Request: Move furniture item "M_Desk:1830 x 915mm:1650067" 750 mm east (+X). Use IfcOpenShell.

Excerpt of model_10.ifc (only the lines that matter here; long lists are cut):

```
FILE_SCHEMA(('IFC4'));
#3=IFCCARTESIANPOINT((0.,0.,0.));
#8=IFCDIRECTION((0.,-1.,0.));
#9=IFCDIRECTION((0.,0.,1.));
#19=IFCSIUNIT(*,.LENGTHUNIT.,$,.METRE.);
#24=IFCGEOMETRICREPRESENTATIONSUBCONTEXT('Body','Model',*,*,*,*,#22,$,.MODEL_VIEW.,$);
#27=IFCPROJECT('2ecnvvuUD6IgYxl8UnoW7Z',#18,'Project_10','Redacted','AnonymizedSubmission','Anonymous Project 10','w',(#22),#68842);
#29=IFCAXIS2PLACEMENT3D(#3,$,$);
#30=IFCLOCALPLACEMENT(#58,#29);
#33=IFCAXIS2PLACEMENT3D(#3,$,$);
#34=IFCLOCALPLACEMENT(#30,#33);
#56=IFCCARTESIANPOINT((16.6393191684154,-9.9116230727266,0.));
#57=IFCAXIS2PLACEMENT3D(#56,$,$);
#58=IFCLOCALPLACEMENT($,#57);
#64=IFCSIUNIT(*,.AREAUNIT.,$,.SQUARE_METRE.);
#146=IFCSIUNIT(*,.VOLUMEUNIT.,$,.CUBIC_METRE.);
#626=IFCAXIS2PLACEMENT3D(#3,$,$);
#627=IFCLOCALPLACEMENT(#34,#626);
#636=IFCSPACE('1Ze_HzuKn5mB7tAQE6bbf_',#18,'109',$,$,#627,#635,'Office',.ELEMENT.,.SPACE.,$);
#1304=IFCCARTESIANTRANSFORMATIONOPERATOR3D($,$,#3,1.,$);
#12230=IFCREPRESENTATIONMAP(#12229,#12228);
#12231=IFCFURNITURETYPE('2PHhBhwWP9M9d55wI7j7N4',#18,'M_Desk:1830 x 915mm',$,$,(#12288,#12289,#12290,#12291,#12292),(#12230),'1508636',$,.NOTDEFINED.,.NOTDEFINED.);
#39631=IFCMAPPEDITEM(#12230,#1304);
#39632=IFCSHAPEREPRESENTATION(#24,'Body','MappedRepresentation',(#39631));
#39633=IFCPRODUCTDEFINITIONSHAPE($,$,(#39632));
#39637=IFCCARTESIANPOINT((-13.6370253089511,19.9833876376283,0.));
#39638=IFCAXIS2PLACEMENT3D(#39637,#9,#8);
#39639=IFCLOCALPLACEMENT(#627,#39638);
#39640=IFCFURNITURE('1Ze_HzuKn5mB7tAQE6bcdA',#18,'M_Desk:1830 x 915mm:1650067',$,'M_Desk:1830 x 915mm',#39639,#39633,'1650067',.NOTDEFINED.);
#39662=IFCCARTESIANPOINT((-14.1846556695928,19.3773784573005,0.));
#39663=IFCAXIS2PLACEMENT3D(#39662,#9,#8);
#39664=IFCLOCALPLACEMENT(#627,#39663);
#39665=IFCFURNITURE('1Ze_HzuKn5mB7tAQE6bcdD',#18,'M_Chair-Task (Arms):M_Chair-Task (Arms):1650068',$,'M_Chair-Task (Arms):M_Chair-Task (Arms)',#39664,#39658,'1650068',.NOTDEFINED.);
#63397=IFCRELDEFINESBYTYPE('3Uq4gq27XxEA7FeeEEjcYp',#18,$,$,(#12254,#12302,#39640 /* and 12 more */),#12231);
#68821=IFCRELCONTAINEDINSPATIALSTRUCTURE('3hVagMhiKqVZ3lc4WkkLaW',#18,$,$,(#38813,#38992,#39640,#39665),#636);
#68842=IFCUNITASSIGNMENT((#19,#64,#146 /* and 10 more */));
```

```python
import ifcopenshell
import ifcopenshell.api.geometry
import ifcopenshell.util.placement

model = ifcopenshell.open("model_10.ifc")

item = model.by_id(39640)
matrix = ifcopenshell.util.placement.get_local_placement(item.ObjectPlacement)
matrix[0, 3] += 0.75
ifcopenshell.api.geometry.edit_object_placement(model, product=item, matrix=matrix, is_si=False)

print(ifcopenshell.util.placement.get_local_placement(item.ObjectPlacement).round(3) + 0.0)

model.write("model_10_v2.ifc")
```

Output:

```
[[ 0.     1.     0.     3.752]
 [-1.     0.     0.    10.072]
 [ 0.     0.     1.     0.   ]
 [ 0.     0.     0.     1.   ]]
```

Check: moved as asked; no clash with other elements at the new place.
